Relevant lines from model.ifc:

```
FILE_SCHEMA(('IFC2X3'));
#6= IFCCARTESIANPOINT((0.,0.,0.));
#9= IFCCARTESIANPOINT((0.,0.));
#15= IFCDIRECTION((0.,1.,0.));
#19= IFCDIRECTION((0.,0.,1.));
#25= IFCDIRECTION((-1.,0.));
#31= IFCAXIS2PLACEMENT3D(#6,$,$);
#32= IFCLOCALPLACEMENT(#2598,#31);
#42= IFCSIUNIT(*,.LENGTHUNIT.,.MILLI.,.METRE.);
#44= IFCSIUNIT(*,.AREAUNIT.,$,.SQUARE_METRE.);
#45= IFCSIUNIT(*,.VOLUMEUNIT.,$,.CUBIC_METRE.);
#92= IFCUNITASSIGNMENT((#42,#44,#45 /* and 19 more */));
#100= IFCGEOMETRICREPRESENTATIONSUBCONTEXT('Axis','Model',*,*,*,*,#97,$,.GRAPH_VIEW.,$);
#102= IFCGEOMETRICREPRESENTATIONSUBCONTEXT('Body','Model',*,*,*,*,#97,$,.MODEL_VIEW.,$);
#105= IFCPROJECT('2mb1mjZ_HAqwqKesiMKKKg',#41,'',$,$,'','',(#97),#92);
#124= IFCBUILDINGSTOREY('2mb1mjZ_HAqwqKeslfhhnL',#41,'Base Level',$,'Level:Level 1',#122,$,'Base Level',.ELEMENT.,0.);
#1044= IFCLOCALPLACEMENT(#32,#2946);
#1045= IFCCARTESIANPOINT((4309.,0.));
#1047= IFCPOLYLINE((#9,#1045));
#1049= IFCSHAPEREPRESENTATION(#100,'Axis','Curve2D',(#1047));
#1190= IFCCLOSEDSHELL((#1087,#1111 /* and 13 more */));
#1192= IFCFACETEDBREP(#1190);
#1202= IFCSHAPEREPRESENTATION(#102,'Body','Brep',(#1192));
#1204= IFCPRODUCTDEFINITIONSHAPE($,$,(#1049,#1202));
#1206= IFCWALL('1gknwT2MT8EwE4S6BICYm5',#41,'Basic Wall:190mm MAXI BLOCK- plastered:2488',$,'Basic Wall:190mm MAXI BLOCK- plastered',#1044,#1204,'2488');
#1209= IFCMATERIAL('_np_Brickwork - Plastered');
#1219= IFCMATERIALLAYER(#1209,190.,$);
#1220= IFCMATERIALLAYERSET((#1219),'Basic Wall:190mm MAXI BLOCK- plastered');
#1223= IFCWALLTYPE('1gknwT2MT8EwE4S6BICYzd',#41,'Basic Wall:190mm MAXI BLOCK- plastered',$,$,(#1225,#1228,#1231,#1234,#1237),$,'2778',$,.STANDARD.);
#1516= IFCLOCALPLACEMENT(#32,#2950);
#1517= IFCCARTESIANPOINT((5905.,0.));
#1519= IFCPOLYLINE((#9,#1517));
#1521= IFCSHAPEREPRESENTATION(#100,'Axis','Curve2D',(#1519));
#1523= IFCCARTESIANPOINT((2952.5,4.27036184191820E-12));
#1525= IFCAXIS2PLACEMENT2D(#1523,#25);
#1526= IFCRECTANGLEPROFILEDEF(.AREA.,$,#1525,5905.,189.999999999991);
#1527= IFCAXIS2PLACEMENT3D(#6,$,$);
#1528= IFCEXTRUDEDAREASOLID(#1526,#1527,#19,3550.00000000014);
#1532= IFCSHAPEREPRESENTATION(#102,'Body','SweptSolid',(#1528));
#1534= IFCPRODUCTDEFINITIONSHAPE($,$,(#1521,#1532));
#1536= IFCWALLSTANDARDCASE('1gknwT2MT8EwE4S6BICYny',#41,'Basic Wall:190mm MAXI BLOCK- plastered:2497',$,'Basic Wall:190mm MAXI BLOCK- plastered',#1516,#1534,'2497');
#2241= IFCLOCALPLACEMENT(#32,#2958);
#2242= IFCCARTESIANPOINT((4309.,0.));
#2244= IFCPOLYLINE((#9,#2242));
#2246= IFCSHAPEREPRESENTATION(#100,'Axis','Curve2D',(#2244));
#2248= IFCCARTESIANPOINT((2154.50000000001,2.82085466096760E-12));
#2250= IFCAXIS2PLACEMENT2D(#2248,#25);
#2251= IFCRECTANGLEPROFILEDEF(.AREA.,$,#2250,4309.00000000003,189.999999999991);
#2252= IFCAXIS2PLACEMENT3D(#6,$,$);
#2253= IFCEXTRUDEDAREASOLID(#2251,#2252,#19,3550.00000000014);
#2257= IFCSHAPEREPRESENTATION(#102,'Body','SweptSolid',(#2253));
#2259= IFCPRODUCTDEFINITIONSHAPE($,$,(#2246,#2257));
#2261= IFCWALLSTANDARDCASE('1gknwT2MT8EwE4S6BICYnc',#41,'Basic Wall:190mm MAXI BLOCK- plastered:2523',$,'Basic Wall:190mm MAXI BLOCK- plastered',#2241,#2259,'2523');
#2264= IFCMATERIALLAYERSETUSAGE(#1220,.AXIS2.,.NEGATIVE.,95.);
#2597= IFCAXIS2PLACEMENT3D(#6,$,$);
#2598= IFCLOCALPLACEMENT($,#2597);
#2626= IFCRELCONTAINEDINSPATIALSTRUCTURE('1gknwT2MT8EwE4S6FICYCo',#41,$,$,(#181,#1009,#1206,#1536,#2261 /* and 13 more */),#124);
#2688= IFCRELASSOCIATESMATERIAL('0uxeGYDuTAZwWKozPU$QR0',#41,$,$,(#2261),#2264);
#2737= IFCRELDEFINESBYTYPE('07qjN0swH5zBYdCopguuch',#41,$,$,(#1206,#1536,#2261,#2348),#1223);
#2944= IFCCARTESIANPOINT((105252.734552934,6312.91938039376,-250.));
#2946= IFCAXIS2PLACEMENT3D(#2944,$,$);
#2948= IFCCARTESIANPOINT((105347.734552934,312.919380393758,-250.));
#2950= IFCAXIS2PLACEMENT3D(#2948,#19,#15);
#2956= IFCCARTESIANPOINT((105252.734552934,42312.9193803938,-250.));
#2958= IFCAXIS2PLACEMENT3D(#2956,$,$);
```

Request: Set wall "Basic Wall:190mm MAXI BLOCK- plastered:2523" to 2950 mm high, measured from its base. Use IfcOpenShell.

```python
import ifcopenshell
import ifcopenshell.geom
import ifcopenshell.util.representation
import ifcopenshell.util.shape
import ifcopenshell.util.unit

model = ifcopenshell.open("model.ifc")
unit_scale = ifcopenshell.util.unit.calculate_unit_scale(model)
settings = ifcopenshell.geom.settings()


def volume(element):
    """Net volume in cubic metres, openings subtracted."""
    shape = ifcopenshell.geom.create_shape(settings, element)
    return ifcopenshell.util.shape.get_volume(shape.geometry)


wall = model.by_guid("1gknwT2MT8EwE4S6BICYnc")
before = volume(wall)

body = ifcopenshell.util.representation.get_representation(wall, "Model", "Body")
solid = body.Items[0]
old_height = solid.Depth
solid.Depth = 2.95 / unit_scale
after = volume(wall)

print(f"height {old_height:g} -> {solid.Depth:g}, volume {before:.3f} -> {after:.3f} m3")

model.write("model_edited.ifc")
```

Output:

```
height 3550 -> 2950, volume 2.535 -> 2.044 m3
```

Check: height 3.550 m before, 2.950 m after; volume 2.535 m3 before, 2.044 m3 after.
